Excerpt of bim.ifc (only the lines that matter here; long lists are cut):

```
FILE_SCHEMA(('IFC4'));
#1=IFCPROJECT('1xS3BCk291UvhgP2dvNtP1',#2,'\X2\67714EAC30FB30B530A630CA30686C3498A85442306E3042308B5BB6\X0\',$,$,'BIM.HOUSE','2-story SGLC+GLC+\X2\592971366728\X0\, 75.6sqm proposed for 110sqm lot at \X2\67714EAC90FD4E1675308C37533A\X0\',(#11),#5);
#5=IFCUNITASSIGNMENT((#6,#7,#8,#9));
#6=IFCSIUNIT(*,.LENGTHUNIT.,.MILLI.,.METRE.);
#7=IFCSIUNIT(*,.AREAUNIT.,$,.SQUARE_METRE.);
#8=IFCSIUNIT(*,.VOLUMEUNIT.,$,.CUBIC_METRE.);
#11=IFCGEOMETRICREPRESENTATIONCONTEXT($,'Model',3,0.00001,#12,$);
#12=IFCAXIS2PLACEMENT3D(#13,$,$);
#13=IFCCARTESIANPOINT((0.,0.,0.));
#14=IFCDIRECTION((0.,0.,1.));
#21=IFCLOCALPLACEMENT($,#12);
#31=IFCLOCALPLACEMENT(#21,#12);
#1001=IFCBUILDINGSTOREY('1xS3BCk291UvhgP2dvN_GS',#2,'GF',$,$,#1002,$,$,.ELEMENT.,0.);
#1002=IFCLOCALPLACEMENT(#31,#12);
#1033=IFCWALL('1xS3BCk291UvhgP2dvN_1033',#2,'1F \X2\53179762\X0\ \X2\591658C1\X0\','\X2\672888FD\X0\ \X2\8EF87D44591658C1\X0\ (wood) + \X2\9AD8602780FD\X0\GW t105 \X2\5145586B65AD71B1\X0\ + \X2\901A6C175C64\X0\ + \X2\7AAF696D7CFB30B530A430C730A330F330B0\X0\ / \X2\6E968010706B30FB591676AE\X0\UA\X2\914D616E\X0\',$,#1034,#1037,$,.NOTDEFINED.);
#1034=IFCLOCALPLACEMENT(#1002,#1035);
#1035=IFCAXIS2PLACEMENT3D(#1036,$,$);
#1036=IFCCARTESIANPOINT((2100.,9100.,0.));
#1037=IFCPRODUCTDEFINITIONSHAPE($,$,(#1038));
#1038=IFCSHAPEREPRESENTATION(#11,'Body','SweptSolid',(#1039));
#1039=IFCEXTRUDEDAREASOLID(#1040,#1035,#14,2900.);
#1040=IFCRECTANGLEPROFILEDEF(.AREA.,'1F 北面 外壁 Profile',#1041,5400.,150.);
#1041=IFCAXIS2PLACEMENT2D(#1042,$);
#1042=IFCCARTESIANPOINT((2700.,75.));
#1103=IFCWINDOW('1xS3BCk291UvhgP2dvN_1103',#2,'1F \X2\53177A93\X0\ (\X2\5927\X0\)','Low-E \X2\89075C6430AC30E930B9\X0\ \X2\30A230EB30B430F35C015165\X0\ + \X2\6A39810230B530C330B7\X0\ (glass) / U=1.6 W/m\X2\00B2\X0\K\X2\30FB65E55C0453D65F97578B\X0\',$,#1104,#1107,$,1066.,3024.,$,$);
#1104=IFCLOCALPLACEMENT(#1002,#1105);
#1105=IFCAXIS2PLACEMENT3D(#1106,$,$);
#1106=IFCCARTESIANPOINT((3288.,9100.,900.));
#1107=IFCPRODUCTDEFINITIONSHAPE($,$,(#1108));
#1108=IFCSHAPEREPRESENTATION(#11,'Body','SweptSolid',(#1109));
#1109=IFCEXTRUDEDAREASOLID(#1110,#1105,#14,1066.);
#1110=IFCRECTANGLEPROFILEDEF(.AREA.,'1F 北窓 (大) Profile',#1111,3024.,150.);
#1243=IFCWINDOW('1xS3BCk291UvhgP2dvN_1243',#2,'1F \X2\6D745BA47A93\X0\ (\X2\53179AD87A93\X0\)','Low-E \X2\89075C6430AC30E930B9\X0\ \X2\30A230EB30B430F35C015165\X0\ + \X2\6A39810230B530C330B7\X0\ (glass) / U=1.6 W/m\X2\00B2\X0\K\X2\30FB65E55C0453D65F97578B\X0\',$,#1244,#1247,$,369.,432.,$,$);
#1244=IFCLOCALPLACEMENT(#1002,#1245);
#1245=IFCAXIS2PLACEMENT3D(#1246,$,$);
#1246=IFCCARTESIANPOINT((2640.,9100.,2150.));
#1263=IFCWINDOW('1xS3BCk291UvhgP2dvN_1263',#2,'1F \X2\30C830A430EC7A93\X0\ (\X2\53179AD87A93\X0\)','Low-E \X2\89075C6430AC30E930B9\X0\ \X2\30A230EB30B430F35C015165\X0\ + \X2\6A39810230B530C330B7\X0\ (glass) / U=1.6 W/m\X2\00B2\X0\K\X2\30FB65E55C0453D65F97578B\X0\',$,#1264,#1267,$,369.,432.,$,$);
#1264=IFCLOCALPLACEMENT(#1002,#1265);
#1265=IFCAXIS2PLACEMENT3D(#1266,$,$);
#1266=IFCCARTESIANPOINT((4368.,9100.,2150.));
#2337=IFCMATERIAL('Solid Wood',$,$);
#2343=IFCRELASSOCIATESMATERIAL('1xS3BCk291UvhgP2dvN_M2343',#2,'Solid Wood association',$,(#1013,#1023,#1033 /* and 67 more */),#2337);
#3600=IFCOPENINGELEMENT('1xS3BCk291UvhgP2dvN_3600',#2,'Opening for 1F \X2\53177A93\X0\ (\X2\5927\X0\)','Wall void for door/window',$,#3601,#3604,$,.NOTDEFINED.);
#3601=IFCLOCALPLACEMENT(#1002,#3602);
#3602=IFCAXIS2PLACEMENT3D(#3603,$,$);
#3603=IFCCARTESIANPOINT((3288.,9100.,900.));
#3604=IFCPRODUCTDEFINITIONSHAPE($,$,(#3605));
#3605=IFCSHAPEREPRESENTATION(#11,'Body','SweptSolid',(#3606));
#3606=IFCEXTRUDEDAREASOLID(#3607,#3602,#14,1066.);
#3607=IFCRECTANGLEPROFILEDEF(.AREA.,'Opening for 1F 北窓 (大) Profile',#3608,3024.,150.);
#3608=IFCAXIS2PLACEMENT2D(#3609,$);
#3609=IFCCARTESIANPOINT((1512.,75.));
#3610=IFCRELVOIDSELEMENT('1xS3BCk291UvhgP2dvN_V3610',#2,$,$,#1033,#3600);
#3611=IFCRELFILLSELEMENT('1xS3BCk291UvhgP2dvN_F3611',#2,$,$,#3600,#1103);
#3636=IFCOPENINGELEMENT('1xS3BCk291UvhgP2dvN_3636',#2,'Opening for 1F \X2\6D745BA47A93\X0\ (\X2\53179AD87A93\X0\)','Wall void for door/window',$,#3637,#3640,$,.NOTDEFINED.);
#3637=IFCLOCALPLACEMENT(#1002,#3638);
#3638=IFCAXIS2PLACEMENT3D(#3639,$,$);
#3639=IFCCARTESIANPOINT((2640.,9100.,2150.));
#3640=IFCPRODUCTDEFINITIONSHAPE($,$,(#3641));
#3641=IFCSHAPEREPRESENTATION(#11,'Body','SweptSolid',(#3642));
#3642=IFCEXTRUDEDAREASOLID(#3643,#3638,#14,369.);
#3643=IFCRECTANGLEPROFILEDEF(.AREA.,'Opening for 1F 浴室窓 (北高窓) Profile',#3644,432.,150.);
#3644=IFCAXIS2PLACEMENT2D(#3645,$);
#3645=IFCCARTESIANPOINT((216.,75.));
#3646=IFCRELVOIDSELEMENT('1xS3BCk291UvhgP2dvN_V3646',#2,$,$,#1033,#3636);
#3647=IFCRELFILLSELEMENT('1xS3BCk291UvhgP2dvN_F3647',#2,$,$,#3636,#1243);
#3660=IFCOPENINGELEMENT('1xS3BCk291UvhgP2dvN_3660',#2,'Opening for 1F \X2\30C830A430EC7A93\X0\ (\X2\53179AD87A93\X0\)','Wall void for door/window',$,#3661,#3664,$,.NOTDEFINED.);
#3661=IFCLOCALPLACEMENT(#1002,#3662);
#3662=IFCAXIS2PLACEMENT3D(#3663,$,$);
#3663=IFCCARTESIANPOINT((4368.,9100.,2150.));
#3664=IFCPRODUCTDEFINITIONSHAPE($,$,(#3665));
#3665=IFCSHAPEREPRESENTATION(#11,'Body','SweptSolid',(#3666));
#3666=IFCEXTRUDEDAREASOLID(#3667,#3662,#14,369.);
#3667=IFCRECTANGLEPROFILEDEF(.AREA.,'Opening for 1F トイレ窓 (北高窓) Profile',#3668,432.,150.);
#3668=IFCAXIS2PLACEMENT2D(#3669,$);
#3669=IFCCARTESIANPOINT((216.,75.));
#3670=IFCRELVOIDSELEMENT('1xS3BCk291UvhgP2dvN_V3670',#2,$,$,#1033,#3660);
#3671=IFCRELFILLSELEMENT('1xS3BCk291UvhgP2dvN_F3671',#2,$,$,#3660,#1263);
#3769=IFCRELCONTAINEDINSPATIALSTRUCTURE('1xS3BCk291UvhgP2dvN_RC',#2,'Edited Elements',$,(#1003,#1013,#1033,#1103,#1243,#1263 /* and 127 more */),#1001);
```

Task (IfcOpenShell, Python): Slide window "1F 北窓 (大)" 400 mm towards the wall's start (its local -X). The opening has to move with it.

```python
import ifcopenshell
import ifcopenshell.api.geometry
import ifcopenshell.util.placement
import ifcopenshell.util.unit

model = ifcopenshell.open("bim.ifc")
unit_scale = ifcopenshell.util.unit.calculate_unit_scale(model)

window = model.by_id(1103)
opening = window.FillsVoids[0].RelatingOpeningElement
wall = opening.VoidsElements[0].RelatingBuildingElement

wall_matrix = ifcopenshell.util.placement.get_local_placement(wall.ObjectPlacement)
shift = wall_matrix[:3, 0] * -0.4 / unit_scale
before = ifcopenshell.util.placement.get_local_placement(window.ObjectPlacement)[:3, 3].copy()

# The window is not placed relative to its opening, so move both.
for product in (opening, window):
    matrix = ifcopenshell.util.placement.get_local_placement(product.ObjectPlacement)
    matrix[:3, 3] += shift
    ifcopenshell.api.geometry.edit_object_placement(model, product=product, matrix=matrix, is_si=False)

after = ifcopenshell.util.placement.get_local_placement(window.ObjectPlacement)[:3, 3]
print("window moved by", (after - before).round(3) + 0.0)

model.write("bim-out.ifc")
```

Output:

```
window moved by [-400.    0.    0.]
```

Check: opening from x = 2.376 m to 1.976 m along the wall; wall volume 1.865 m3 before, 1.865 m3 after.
